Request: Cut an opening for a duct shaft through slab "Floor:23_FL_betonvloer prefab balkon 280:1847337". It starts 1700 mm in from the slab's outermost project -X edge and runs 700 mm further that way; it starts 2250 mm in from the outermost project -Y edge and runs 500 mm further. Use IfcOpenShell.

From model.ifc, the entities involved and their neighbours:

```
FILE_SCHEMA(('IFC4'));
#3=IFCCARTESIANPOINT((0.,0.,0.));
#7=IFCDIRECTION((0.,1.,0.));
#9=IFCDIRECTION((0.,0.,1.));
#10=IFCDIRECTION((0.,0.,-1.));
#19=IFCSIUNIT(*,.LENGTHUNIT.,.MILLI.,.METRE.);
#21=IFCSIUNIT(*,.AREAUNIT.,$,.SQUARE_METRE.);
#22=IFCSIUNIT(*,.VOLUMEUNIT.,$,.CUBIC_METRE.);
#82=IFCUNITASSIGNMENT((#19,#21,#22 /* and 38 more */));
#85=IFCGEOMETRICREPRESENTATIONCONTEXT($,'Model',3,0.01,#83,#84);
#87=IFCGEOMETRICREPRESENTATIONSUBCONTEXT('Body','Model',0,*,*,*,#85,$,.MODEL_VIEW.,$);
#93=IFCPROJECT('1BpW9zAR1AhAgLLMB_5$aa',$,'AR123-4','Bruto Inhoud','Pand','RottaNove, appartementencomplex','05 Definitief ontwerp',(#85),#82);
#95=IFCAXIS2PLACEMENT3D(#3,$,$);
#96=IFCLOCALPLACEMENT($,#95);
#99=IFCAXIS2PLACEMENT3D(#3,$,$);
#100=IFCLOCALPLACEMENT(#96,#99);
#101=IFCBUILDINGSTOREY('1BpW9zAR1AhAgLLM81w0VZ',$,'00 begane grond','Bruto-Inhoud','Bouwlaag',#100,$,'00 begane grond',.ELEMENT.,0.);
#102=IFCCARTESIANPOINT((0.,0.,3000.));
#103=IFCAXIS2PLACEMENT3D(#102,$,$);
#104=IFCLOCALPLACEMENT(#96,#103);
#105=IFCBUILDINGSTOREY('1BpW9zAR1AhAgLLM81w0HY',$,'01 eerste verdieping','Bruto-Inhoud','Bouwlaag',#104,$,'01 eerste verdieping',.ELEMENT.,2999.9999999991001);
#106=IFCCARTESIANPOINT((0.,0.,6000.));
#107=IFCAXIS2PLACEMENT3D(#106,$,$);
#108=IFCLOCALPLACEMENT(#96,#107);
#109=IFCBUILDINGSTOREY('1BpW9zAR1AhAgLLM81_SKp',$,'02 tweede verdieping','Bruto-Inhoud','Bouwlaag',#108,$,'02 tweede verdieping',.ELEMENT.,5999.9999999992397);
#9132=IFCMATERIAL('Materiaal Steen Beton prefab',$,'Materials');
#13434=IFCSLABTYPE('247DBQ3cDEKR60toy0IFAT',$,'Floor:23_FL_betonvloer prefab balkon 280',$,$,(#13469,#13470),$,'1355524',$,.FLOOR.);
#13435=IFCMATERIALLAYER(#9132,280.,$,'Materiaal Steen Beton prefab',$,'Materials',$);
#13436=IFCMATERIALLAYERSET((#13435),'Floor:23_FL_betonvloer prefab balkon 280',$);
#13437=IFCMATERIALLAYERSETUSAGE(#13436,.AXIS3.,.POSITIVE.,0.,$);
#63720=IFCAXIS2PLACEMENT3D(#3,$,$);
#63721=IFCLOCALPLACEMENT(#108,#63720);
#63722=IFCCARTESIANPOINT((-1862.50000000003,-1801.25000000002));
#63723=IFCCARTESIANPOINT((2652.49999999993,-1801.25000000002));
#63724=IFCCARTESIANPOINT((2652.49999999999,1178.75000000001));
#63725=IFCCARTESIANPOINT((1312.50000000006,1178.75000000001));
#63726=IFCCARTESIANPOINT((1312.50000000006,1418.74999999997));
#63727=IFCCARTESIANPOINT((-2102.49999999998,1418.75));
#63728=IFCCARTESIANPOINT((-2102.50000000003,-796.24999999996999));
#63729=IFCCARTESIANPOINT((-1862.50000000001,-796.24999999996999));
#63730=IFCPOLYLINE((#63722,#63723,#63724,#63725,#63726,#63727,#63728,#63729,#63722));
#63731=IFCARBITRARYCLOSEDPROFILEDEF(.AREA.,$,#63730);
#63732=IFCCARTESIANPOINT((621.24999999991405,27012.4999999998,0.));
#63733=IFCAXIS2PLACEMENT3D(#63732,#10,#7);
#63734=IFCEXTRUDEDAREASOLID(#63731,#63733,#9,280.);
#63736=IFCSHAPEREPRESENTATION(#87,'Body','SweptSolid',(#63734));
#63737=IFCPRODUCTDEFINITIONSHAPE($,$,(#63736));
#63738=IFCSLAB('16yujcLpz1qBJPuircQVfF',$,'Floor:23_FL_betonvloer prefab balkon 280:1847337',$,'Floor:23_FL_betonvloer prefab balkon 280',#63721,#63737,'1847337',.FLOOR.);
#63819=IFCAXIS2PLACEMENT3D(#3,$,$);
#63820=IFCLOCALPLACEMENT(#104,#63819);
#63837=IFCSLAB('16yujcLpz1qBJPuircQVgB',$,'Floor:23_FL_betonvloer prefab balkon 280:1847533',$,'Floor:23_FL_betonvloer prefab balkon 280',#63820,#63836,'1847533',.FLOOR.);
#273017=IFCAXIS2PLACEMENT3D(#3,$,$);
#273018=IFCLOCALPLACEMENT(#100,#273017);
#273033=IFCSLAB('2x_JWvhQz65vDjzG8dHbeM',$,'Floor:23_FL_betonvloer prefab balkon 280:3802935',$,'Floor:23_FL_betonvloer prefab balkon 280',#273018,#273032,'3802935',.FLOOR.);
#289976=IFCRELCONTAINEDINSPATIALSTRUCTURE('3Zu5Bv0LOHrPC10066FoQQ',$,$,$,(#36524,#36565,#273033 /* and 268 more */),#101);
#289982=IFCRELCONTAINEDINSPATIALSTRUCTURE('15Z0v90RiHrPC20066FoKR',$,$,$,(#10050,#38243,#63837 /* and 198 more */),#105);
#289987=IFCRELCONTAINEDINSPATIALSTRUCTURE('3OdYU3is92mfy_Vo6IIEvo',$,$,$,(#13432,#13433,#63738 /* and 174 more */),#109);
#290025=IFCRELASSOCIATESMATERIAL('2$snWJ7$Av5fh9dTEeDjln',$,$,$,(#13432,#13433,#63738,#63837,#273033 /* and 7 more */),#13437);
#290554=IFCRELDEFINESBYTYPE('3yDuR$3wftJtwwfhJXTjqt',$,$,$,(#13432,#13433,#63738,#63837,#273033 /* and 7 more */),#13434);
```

```python
import numpy as np
import ifcopenshell
import ifcopenshell.api.feature
import ifcopenshell.api.geometry
import ifcopenshell.api.root
import ifcopenshell.geom
import ifcopenshell.util.placement
import ifcopenshell.util.representation
import ifcopenshell.util.shape
import ifcopenshell.util.unit

model = ifcopenshell.open("model.ifc")
unit_scale = ifcopenshell.util.unit.calculate_unit_scale(model)
settings = ifcopenshell.geom.settings()


def volume(element):
    """Net volume in cubic metres, openings subtracted."""
    shape = ifcopenshell.geom.create_shape(settings, element)
    return ifcopenshell.util.shape.get_volume(shape.geometry)


slab = model.by_id(63738)
before = volume(slab)

# Extent in the slab's own axes, in metres. The edges named are its -X and -Y sides.
slab_shape = ifcopenshell.geom.create_shape(settings, slab)
vertices = ifcopenshell.util.shape.get_vertices(slab_shape.geometry)
x_min, y_min, bottom = vertices.min(axis=0)
top = vertices[:, 2].max()

opening = ifcopenshell.api.root.create_entity(model, ifc_class="IfcOpeningElement", name="Duct shaft opening", predefined_type="OPENING")
context = ifcopenshell.util.representation.get_context(model, "Model", "Body", "MODEL_VIEW")
width, depth = 0.7, 0.5
outline = [(0.0, 0.0), (width, 0.0), (width, depth), (0.0, depth), (0.0, 0.0)]
# Overshoot both faces by 50 mm so the cut is clean.
shape = ifcopenshell.api.geometry.add_slab_representation(
    model, context=context, depth=top - bottom + 0.1, polyline=outline
)
ifcopenshell.api.geometry.assign_representation(model, product=opening, representation=shape)

matrix = ifcopenshell.util.placement.get_local_placement(slab.ObjectPlacement)
matrix[:, 3] = matrix @ np.append(np.array([x_min + 1.7, y_min + 2.25, bottom - 0.05]) / unit_scale, 1.0)
ifcopenshell.api.geometry.edit_object_placement(model, product=opening, matrix=matrix, is_si=False)
ifcopenshell.api.feature.add_feature(model, feature=opening, element=slab)

after = volume(slab)

print(f"slab volume {before:.3f} -> {after:.3f} m3")

model.write("model_updated.ifc")
```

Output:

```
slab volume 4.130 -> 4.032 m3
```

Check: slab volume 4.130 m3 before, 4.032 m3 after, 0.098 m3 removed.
